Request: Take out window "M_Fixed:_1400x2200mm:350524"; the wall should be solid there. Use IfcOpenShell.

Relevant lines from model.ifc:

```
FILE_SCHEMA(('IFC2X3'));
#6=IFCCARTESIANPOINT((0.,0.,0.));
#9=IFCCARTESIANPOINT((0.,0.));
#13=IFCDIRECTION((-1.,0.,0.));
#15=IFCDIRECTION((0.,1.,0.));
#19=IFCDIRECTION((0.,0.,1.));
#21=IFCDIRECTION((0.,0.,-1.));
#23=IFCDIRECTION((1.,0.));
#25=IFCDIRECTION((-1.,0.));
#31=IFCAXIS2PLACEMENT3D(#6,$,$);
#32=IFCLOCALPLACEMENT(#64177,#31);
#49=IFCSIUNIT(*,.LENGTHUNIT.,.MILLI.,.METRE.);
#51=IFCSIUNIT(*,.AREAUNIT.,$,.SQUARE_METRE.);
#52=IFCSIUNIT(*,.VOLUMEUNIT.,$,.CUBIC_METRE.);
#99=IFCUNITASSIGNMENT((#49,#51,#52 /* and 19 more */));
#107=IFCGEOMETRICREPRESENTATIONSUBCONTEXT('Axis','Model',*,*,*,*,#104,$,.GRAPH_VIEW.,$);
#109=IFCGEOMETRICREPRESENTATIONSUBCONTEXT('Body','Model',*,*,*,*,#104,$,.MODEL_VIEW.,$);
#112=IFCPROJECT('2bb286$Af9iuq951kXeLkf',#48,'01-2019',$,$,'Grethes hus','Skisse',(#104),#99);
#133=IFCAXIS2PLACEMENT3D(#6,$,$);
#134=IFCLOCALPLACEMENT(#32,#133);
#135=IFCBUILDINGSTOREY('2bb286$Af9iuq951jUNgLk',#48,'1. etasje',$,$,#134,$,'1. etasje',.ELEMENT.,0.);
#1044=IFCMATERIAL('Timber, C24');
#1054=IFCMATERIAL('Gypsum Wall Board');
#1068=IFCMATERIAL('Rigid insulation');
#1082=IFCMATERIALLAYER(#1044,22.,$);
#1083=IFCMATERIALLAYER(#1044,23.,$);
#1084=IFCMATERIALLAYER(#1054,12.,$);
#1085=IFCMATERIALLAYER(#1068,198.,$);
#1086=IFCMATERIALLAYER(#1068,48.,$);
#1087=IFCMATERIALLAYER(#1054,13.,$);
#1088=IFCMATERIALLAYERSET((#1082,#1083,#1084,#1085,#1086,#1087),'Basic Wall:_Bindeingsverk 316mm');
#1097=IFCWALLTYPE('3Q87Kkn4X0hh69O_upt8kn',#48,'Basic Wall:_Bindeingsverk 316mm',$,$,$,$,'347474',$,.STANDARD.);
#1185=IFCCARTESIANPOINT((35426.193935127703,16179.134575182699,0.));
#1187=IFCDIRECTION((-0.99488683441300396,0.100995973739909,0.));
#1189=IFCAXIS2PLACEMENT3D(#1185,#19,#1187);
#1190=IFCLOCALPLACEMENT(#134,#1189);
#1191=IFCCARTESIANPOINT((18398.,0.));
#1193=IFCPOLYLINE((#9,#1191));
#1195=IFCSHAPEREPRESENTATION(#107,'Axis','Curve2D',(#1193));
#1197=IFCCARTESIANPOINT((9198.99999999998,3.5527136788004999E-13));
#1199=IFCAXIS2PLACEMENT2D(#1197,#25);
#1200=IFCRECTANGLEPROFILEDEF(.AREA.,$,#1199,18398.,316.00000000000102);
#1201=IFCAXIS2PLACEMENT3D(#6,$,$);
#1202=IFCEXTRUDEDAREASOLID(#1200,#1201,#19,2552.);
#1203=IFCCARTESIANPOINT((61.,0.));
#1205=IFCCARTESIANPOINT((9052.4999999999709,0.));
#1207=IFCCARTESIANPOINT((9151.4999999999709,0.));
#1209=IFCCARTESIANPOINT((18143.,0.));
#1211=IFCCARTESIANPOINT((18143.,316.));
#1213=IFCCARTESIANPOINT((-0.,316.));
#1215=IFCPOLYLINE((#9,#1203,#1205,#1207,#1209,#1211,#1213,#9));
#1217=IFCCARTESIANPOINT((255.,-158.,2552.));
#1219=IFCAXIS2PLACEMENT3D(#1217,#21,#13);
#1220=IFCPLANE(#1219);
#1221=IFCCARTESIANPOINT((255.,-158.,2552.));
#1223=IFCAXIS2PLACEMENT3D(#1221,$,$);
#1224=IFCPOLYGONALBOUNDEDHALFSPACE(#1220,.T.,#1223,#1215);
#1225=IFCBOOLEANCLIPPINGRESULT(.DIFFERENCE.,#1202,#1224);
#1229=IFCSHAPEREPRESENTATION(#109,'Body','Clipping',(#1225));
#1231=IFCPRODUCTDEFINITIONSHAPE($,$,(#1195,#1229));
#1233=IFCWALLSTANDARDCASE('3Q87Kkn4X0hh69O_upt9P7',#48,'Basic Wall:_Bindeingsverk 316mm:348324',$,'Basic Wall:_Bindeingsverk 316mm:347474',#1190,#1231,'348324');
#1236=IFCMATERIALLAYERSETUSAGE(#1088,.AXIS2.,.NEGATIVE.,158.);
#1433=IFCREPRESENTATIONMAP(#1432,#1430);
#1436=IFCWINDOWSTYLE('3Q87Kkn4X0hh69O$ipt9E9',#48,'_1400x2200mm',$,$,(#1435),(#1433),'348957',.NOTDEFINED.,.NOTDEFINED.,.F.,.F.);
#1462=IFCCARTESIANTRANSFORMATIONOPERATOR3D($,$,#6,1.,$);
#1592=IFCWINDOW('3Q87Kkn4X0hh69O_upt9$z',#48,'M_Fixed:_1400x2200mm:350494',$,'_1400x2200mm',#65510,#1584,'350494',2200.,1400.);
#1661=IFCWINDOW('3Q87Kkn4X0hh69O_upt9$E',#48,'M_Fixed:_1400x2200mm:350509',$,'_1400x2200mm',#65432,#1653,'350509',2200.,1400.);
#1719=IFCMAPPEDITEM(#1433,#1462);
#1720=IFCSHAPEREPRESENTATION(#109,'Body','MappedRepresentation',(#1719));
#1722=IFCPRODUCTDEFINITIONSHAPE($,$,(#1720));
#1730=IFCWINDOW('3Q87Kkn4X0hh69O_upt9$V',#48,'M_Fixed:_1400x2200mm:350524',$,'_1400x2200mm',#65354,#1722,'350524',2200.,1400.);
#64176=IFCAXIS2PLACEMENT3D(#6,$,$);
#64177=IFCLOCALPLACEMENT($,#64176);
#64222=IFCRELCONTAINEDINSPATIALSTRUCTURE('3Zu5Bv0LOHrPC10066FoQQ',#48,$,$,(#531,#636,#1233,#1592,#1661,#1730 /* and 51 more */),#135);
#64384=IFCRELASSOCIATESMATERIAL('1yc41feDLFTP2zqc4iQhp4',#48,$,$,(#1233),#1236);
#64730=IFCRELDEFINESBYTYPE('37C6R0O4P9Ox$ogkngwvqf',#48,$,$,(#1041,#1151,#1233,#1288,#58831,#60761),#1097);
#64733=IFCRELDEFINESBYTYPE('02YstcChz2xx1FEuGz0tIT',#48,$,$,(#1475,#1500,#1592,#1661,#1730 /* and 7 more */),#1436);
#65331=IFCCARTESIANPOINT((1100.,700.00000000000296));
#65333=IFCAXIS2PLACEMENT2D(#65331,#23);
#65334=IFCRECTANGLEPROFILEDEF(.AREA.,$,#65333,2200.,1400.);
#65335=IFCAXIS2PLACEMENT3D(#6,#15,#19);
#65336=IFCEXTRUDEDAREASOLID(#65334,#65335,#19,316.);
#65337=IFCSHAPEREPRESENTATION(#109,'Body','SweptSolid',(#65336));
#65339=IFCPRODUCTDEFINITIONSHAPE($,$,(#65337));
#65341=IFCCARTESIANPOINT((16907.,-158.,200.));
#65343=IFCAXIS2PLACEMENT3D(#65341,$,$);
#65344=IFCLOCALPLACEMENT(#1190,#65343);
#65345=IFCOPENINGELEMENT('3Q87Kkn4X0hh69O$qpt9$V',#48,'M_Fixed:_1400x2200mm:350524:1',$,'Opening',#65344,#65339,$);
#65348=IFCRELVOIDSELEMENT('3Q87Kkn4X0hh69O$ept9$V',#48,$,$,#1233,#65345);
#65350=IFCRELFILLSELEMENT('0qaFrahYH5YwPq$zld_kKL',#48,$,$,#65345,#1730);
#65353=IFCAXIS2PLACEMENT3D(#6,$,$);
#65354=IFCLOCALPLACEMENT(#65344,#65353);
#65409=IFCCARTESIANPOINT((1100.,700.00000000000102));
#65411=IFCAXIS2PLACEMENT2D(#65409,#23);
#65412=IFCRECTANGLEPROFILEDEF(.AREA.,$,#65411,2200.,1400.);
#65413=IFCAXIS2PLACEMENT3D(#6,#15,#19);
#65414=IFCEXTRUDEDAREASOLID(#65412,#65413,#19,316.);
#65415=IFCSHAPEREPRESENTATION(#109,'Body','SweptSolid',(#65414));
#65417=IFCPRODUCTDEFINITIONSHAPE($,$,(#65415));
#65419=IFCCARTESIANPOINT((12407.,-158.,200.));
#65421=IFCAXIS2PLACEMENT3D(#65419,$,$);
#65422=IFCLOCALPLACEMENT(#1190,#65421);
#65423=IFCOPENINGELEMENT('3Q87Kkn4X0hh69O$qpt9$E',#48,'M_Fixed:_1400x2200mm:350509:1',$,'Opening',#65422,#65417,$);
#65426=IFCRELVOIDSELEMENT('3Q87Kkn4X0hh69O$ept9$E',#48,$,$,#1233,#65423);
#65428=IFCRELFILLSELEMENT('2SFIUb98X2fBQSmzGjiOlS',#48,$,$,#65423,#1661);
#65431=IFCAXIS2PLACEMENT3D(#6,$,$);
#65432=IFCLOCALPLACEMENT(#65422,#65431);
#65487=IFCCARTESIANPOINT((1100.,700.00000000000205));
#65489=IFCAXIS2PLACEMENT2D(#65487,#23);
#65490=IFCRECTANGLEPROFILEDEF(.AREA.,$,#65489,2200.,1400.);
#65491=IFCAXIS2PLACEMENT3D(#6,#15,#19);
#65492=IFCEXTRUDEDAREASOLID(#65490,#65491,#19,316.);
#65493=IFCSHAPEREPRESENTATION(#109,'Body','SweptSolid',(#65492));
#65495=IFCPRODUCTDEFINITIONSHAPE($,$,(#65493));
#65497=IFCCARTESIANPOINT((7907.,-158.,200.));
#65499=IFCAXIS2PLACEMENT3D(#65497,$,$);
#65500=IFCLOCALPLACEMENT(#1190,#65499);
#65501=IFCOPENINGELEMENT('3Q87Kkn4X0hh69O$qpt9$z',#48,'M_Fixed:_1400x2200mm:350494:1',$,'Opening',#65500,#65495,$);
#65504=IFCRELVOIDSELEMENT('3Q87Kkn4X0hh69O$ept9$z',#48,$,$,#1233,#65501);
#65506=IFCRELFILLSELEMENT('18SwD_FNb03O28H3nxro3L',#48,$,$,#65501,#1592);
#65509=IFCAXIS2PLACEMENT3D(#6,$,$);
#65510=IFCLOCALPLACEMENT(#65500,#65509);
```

```python
import ifcopenshell
import ifcopenshell.api.feature
import ifcopenshell.api.root
import ifcopenshell.geom
import ifcopenshell.util.shape

model = ifcopenshell.open("model.ifc")
settings = ifcopenshell.geom.settings()


def volume(element):
    """Net volume in cubic metres, openings subtracted."""
    shape = ifcopenshell.geom.create_shape(settings, element)
    return ifcopenshell.util.shape.get_volume(shape.geometry)


window = model.by_guid("3Q87Kkn4X0hh69O_upt9$V")
opening = window.FillsVoids[0].RelatingOpeningElement
wall = opening.VoidsElements[0].RelatingBuildingElement
before = volume(wall)

ifcopenshell.api.root.remove_product(model, product=window)
ifcopenshell.api.feature.remove_feature(model, feature=opening)

after = volume(wall)

print(f"wall volume {before:.3f} -> {after:.3f} m3")

model.write("model_v2.ifc")
```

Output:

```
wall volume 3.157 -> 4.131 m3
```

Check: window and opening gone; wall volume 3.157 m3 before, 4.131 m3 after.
